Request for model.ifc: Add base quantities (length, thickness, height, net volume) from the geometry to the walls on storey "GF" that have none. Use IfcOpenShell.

First a look at what the model holds.

```python
import ifcopenshell
import ifcopenshell.util.element
import ifcopenshell.util.unit

model = ifcopenshell.open("model.ifc")
print(model.schema)
for unit_type in ("LENGTHUNIT", "AREAUNIT", "VOLUMEUNIT"):
    print(unit_type, ifcopenshell.util.unit.calculate_unit_scale(model, unit_type))
storey = next(s for s in model.by_type("IfcBuildingStorey") if s.Name == "GF")
walls = [e for e in ifcopenshell.util.element.get_decomposition(storey) if e.is_a("IfcWall")]
for e in sorted(walls, key=lambda e: e.id()):
    print(e.id(), e.is_a(), e.Name, list(ifcopenshell.util.element.get_psets(e, qtos_only=True)), sep=" | ")
```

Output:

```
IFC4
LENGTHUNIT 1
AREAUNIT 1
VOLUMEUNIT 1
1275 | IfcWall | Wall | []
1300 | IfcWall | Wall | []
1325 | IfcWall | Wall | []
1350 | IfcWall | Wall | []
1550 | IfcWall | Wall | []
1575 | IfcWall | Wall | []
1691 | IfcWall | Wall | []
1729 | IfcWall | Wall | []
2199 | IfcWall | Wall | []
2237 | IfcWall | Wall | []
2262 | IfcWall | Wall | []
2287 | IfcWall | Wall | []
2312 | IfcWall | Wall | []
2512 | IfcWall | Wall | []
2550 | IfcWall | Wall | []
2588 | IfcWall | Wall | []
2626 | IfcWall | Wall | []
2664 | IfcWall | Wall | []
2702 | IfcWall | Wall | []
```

```python
import ifcopenshell
import ifcopenshell.api.pset
import ifcopenshell.geom
import ifcopenshell.util.element
import ifcopenshell.util.shape
import ifcopenshell.util.unit

model = ifcopenshell.open("model.ifc")
unit_scale = ifcopenshell.util.unit.calculate_unit_scale(model)
volume_scale = ifcopenshell.util.unit.calculate_unit_scale(model, "VOLUMEUNIT")
settings = ifcopenshell.geom.settings()

storey = next(s for s in model.by_type("IfcBuildingStorey") if s.Name == "GF")
walls = [e for e in ifcopenshell.util.element.get_decomposition(storey) if e.is_a("IfcWall")]

for e in sorted(walls, key=lambda e: e.id()):
    if ifcopenshell.util.element.get_psets(e, qtos_only=True, should_inherit=False):
        continue
    # Geometry comes back in metres, in the element's own axes.
    shape = ifcopenshell.geom.create_shape(settings, e)
    values = {
        "Length": ifcopenshell.util.shape.get_x(shape.geometry) / unit_scale,
        "Width": ifcopenshell.util.shape.get_y(shape.geometry) / unit_scale,
        "Height": ifcopenshell.util.shape.get_z(shape.geometry) / unit_scale,
        "NetVolume": ifcopenshell.util.shape.get_volume(shape.geometry) / volume_scale,
    }
    qto = ifcopenshell.api.pset.add_qto(model, product=e, name="Qto_WallBaseQuantities")
    ifcopenshell.api.pset.edit_qto(model, qto=qto, properties=values)
    print(e.id(), {k: round(v, 3) for k, v in values.items()})

model.write("model_edited.ifc")
```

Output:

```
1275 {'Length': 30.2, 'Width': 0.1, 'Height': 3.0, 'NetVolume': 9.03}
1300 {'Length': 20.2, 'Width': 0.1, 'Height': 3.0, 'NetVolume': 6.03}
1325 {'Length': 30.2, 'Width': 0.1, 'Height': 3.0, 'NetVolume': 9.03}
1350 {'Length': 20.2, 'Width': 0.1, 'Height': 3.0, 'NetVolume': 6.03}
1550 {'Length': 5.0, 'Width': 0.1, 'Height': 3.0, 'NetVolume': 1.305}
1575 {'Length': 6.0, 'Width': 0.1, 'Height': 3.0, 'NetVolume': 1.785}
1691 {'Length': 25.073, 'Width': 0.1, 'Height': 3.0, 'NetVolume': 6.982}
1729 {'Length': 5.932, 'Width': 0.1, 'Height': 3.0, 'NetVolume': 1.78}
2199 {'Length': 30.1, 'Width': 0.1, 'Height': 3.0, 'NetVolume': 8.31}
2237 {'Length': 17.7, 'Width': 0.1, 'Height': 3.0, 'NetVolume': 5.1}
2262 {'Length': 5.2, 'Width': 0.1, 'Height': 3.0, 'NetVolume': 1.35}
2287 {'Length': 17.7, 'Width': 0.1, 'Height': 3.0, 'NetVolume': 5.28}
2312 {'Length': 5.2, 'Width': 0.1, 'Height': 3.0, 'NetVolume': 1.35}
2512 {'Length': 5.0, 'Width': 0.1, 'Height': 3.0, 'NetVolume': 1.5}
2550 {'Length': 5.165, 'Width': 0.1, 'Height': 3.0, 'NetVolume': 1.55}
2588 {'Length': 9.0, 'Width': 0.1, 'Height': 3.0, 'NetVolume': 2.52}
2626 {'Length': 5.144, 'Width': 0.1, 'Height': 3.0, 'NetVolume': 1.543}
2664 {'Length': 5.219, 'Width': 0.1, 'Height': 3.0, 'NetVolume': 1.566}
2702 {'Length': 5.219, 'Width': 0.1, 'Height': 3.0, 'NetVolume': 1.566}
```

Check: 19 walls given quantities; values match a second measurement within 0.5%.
